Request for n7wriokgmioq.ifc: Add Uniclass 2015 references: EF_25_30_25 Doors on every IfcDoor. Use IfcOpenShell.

First a look at what the model holds.

```python
import ifcopenshell

model = ifcopenshell.open("n7wriokgmioq.ifc")
print(model.schema)
print("classifications:", [c.Name for c in model.by_type("IfcClassification")])
for ifc_class in ("IfcDoor", "IfcRoof", "IfcStair", "IfcWall", "IfcWindow"):
    print(ifc_class, len(model.by_type(ifc_class)))
```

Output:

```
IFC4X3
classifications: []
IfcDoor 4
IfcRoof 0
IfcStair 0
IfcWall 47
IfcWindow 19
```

```python
import ifcopenshell
import ifcopenshell.api.classification

model = ifcopenshell.open("n7wriokgmioq.ifc")

system = ifcopenshell.api.classification.add_classification(model, classification="Uniclass 2015")

codes = {
    "IfcDoor": ("EF_25_30_25", "Doors"),
}
for ifc_class, (code, name) in codes.items():
    products = model.by_type(ifc_class)
    ifcopenshell.api.classification.add_reference(
        model, products=products, classification=system, identification=code, name=name
    )
    print(code, len(products))

model.write("n7wriokgmioq-out.ifc")
```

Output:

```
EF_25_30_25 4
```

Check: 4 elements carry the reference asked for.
